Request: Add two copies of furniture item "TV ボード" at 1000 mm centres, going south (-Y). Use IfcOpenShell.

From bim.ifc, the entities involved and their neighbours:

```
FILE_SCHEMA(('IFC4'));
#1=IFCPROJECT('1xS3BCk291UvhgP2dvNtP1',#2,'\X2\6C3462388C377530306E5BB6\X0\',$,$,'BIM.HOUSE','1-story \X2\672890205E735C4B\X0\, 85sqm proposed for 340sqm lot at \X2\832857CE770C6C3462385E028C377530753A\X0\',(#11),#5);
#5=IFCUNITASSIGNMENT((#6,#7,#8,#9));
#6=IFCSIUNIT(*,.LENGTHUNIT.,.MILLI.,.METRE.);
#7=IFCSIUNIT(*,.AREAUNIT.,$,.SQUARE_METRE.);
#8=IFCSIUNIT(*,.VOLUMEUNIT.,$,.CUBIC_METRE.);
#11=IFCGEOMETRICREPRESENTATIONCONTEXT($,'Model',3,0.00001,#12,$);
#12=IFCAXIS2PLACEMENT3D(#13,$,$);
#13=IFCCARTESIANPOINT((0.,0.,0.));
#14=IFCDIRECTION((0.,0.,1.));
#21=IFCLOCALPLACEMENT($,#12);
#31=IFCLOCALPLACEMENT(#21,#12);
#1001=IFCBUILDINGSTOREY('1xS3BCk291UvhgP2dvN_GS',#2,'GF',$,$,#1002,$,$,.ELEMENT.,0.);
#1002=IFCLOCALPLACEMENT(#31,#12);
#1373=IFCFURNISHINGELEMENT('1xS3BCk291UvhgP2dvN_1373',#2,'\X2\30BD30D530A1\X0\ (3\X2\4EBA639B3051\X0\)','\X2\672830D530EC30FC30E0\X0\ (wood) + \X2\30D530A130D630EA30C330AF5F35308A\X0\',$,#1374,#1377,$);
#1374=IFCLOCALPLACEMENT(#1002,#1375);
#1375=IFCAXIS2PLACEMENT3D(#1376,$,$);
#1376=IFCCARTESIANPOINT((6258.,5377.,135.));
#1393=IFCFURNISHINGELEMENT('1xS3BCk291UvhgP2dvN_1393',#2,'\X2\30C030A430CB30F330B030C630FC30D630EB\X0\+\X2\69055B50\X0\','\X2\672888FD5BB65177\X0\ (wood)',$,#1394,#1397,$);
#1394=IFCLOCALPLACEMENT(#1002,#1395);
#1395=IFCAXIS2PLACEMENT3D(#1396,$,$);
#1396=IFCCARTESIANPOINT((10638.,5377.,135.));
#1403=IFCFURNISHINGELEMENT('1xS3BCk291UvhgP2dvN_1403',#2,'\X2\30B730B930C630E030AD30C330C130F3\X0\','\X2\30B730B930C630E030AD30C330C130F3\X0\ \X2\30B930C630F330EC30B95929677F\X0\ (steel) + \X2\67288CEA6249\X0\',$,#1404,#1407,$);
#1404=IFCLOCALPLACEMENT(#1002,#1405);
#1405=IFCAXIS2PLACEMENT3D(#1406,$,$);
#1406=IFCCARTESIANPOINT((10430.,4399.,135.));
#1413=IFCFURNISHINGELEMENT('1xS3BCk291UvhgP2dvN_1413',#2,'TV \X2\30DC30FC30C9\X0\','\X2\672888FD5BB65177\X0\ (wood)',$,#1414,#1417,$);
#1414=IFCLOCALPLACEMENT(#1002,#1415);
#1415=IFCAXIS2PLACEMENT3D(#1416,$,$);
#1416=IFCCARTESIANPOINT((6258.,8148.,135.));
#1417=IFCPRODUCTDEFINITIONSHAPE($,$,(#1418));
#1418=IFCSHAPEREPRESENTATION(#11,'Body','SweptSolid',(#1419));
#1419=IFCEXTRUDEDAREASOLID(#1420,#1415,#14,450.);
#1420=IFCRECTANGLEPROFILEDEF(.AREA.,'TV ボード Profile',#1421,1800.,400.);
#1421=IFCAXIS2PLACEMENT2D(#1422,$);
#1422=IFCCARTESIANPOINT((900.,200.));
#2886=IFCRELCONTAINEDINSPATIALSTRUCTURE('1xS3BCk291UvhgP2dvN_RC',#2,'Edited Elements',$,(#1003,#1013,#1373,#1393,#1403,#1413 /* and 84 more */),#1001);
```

```python
import numpy as np
import ifcopenshell
import ifcopenshell.api.geometry
import ifcopenshell.api.root
import ifcopenshell.util.element
import ifcopenshell.util.placement
import ifcopenshell.util.unit

model = ifcopenshell.open("bim.ifc")
unit_scale = ifcopenshell.util.unit.calculate_unit_scale(model)


def reuse_history(source, copy):
    """copy_class also copies each property set's owner history, people and application; keep the originals."""
    for rel in copy.IsDefinedBy:
        if rel.is_a("IfcRelDefinesByProperties") and (history := rel.RelatingPropertyDefinition.OwnerHistory):
            rel.RelatingPropertyDefinition.OwnerHistory = source.OwnerHistory
            ifcopenshell.util.element.remove_deep2(model, history)


source = model.by_guid("1xS3BCk291UvhgP2dvN_1413")
base = ifcopenshell.util.placement.get_local_placement(source.ObjectPlacement)
step = np.array([0.0, -1.0, 0.0]) * 1 / unit_scale

for i in range(1, 3):
    copy = ifcopenshell.api.root.copy_class(model, product=source)
    copy.Representation = ifcopenshell.util.element.copy_deep(
        model, source.Representation, exclude=["IfcGeometricRepresentationContext", "IfcRepresentationMap"]
    )
    reuse_history(source, copy)
    matrix = base.copy()
    matrix[:3, 3] += i * step
    print("added at", matrix[:3, 3].round(3) + 0.0)
    ifcopenshell.api.geometry.edit_object_placement(model, product=copy, matrix=matrix, is_si=False)

model.write("bim-out.ifc")
```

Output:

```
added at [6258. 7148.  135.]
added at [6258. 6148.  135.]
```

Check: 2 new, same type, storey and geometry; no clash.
